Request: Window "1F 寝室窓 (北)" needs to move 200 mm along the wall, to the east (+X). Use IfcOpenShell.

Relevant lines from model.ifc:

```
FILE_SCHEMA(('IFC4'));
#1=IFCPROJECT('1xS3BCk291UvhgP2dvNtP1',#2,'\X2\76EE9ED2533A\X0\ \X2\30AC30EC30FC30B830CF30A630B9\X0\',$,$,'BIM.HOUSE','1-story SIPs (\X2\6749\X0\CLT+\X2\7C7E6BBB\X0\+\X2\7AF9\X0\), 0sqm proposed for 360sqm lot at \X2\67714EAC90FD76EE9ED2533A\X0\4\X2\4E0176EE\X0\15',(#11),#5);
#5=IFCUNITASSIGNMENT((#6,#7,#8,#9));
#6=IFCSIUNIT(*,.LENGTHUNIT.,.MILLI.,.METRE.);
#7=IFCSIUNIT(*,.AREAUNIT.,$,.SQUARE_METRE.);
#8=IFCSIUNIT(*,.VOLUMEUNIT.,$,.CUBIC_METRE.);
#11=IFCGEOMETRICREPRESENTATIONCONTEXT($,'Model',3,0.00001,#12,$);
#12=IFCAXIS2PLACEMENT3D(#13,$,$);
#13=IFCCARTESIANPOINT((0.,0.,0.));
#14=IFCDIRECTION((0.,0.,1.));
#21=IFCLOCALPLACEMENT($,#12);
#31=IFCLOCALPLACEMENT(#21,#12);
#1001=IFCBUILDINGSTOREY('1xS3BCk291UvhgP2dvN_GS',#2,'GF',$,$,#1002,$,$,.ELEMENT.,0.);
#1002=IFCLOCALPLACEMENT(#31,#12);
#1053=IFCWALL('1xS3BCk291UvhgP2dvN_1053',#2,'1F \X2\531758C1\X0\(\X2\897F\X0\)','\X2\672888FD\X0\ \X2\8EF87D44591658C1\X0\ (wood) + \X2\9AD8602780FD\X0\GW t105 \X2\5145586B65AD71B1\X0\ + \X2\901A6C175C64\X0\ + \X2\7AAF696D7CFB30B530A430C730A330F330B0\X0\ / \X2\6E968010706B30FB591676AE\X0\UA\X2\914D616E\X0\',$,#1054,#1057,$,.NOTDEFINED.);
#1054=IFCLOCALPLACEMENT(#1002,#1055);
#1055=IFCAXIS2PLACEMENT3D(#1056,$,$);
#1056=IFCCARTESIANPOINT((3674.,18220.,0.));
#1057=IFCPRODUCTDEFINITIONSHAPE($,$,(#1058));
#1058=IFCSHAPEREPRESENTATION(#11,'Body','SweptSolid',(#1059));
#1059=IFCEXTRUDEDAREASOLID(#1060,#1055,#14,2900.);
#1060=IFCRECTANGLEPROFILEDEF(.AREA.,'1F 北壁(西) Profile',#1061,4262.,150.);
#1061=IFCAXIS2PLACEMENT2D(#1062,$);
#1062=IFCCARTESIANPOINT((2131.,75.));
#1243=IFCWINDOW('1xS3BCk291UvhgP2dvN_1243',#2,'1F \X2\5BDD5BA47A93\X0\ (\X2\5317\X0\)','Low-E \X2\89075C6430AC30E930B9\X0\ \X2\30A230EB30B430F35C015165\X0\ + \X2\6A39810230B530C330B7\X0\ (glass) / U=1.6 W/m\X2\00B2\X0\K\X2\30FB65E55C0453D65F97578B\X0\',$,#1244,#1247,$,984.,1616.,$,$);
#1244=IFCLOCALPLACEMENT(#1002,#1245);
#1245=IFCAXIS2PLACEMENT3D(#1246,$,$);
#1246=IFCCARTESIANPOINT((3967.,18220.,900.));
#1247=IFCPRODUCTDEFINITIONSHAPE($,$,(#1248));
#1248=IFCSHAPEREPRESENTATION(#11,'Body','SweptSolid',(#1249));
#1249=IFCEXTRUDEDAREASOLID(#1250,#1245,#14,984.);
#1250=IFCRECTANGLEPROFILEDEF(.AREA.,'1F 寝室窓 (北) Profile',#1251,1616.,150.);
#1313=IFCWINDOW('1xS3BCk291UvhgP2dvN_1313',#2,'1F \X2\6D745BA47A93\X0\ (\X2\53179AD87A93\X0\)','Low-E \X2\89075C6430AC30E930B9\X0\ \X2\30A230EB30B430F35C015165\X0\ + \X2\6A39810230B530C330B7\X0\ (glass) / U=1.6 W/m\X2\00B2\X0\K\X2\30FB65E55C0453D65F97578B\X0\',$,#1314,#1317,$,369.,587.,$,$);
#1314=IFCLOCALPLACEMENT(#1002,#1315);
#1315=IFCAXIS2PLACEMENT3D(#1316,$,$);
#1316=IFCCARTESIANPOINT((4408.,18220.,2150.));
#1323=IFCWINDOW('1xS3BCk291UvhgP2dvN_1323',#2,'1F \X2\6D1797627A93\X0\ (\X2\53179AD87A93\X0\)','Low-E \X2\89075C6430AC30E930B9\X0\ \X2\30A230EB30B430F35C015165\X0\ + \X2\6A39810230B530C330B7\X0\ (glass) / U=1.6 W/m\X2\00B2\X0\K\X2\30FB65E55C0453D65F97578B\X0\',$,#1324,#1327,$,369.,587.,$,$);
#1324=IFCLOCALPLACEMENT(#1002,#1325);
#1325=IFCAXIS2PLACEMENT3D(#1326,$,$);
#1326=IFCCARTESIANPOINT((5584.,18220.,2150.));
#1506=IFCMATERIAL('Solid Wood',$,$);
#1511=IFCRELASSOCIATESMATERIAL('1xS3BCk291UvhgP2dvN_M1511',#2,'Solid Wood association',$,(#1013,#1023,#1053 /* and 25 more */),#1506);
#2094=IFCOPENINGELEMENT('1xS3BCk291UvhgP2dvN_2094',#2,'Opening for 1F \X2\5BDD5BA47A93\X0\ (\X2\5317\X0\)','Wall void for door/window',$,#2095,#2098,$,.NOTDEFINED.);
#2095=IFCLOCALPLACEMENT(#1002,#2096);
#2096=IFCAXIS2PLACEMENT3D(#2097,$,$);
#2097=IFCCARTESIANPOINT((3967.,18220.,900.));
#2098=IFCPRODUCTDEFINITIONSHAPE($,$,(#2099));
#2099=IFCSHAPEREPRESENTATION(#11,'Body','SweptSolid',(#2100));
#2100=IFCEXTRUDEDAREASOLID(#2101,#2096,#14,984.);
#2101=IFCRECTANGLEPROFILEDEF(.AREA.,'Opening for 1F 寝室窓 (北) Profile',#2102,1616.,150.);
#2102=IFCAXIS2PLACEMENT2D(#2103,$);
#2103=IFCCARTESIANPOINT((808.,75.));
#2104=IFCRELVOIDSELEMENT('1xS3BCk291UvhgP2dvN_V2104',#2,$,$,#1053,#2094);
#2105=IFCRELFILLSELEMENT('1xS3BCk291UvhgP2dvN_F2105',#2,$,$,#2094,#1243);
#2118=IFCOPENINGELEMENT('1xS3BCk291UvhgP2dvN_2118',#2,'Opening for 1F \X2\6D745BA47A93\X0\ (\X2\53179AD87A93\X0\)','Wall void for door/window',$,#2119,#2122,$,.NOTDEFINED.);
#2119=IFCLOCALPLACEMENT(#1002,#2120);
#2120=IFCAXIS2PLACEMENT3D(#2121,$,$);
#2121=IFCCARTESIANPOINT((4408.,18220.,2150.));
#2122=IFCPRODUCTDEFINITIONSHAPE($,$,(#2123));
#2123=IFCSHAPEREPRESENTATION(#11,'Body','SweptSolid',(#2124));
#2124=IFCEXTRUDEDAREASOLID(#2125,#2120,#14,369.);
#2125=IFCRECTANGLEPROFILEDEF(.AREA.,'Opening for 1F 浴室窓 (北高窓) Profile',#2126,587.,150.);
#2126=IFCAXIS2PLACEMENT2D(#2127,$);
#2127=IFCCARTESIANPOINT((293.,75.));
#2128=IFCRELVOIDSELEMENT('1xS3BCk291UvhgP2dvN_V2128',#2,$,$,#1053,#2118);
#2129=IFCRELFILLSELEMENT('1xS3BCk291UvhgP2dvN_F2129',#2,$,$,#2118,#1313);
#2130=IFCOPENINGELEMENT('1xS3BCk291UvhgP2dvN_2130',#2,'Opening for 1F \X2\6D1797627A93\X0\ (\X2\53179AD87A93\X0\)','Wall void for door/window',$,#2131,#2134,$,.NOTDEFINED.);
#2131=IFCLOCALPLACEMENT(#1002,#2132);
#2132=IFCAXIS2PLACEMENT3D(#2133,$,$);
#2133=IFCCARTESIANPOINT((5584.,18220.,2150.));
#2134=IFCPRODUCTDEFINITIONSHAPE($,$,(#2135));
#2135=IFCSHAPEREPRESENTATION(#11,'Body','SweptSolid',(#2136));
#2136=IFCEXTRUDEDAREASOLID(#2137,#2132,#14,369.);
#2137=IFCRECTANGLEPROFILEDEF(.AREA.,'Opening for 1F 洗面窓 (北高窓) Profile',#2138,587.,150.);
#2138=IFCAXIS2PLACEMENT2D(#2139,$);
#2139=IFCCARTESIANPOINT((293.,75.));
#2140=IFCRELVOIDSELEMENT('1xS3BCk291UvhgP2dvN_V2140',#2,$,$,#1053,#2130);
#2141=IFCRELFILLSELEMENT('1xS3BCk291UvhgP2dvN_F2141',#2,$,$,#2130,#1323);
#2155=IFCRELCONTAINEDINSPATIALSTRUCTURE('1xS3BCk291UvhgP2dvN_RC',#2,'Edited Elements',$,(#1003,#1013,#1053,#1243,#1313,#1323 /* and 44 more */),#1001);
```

```python
import ifcopenshell
import ifcopenshell.api.geometry
import ifcopenshell.util.placement
import ifcopenshell.util.unit

model = ifcopenshell.open("model.ifc")
unit_scale = ifcopenshell.util.unit.calculate_unit_scale(model)

window = model.by_guid("1xS3BCk291UvhgP2dvN_1243")
opening = window.FillsVoids[0].RelatingOpeningElement
wall = opening.VoidsElements[0].RelatingBuildingElement

wall_matrix = ifcopenshell.util.placement.get_local_placement(wall.ObjectPlacement)
shift = wall_matrix[:3, 0] * 0.2 / unit_scale
before = ifcopenshell.util.placement.get_local_placement(window.ObjectPlacement)[:3, 3].copy()

# The window is not placed relative to its opening, so move both.
for product in (opening, window):
    matrix = ifcopenshell.util.placement.get_local_placement(product.ObjectPlacement)
    matrix[:3, 3] += shift
    ifcopenshell.api.geometry.edit_object_placement(model, product=product, matrix=matrix, is_si=False)

after = ifcopenshell.util.placement.get_local_placement(window.ObjectPlacement)[:3, 3]
print("window moved by", (after - before).round(3) + 0.0)

model.write("model_updated.ifc")
```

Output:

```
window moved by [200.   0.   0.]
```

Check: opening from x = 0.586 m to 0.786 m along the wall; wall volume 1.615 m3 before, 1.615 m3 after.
